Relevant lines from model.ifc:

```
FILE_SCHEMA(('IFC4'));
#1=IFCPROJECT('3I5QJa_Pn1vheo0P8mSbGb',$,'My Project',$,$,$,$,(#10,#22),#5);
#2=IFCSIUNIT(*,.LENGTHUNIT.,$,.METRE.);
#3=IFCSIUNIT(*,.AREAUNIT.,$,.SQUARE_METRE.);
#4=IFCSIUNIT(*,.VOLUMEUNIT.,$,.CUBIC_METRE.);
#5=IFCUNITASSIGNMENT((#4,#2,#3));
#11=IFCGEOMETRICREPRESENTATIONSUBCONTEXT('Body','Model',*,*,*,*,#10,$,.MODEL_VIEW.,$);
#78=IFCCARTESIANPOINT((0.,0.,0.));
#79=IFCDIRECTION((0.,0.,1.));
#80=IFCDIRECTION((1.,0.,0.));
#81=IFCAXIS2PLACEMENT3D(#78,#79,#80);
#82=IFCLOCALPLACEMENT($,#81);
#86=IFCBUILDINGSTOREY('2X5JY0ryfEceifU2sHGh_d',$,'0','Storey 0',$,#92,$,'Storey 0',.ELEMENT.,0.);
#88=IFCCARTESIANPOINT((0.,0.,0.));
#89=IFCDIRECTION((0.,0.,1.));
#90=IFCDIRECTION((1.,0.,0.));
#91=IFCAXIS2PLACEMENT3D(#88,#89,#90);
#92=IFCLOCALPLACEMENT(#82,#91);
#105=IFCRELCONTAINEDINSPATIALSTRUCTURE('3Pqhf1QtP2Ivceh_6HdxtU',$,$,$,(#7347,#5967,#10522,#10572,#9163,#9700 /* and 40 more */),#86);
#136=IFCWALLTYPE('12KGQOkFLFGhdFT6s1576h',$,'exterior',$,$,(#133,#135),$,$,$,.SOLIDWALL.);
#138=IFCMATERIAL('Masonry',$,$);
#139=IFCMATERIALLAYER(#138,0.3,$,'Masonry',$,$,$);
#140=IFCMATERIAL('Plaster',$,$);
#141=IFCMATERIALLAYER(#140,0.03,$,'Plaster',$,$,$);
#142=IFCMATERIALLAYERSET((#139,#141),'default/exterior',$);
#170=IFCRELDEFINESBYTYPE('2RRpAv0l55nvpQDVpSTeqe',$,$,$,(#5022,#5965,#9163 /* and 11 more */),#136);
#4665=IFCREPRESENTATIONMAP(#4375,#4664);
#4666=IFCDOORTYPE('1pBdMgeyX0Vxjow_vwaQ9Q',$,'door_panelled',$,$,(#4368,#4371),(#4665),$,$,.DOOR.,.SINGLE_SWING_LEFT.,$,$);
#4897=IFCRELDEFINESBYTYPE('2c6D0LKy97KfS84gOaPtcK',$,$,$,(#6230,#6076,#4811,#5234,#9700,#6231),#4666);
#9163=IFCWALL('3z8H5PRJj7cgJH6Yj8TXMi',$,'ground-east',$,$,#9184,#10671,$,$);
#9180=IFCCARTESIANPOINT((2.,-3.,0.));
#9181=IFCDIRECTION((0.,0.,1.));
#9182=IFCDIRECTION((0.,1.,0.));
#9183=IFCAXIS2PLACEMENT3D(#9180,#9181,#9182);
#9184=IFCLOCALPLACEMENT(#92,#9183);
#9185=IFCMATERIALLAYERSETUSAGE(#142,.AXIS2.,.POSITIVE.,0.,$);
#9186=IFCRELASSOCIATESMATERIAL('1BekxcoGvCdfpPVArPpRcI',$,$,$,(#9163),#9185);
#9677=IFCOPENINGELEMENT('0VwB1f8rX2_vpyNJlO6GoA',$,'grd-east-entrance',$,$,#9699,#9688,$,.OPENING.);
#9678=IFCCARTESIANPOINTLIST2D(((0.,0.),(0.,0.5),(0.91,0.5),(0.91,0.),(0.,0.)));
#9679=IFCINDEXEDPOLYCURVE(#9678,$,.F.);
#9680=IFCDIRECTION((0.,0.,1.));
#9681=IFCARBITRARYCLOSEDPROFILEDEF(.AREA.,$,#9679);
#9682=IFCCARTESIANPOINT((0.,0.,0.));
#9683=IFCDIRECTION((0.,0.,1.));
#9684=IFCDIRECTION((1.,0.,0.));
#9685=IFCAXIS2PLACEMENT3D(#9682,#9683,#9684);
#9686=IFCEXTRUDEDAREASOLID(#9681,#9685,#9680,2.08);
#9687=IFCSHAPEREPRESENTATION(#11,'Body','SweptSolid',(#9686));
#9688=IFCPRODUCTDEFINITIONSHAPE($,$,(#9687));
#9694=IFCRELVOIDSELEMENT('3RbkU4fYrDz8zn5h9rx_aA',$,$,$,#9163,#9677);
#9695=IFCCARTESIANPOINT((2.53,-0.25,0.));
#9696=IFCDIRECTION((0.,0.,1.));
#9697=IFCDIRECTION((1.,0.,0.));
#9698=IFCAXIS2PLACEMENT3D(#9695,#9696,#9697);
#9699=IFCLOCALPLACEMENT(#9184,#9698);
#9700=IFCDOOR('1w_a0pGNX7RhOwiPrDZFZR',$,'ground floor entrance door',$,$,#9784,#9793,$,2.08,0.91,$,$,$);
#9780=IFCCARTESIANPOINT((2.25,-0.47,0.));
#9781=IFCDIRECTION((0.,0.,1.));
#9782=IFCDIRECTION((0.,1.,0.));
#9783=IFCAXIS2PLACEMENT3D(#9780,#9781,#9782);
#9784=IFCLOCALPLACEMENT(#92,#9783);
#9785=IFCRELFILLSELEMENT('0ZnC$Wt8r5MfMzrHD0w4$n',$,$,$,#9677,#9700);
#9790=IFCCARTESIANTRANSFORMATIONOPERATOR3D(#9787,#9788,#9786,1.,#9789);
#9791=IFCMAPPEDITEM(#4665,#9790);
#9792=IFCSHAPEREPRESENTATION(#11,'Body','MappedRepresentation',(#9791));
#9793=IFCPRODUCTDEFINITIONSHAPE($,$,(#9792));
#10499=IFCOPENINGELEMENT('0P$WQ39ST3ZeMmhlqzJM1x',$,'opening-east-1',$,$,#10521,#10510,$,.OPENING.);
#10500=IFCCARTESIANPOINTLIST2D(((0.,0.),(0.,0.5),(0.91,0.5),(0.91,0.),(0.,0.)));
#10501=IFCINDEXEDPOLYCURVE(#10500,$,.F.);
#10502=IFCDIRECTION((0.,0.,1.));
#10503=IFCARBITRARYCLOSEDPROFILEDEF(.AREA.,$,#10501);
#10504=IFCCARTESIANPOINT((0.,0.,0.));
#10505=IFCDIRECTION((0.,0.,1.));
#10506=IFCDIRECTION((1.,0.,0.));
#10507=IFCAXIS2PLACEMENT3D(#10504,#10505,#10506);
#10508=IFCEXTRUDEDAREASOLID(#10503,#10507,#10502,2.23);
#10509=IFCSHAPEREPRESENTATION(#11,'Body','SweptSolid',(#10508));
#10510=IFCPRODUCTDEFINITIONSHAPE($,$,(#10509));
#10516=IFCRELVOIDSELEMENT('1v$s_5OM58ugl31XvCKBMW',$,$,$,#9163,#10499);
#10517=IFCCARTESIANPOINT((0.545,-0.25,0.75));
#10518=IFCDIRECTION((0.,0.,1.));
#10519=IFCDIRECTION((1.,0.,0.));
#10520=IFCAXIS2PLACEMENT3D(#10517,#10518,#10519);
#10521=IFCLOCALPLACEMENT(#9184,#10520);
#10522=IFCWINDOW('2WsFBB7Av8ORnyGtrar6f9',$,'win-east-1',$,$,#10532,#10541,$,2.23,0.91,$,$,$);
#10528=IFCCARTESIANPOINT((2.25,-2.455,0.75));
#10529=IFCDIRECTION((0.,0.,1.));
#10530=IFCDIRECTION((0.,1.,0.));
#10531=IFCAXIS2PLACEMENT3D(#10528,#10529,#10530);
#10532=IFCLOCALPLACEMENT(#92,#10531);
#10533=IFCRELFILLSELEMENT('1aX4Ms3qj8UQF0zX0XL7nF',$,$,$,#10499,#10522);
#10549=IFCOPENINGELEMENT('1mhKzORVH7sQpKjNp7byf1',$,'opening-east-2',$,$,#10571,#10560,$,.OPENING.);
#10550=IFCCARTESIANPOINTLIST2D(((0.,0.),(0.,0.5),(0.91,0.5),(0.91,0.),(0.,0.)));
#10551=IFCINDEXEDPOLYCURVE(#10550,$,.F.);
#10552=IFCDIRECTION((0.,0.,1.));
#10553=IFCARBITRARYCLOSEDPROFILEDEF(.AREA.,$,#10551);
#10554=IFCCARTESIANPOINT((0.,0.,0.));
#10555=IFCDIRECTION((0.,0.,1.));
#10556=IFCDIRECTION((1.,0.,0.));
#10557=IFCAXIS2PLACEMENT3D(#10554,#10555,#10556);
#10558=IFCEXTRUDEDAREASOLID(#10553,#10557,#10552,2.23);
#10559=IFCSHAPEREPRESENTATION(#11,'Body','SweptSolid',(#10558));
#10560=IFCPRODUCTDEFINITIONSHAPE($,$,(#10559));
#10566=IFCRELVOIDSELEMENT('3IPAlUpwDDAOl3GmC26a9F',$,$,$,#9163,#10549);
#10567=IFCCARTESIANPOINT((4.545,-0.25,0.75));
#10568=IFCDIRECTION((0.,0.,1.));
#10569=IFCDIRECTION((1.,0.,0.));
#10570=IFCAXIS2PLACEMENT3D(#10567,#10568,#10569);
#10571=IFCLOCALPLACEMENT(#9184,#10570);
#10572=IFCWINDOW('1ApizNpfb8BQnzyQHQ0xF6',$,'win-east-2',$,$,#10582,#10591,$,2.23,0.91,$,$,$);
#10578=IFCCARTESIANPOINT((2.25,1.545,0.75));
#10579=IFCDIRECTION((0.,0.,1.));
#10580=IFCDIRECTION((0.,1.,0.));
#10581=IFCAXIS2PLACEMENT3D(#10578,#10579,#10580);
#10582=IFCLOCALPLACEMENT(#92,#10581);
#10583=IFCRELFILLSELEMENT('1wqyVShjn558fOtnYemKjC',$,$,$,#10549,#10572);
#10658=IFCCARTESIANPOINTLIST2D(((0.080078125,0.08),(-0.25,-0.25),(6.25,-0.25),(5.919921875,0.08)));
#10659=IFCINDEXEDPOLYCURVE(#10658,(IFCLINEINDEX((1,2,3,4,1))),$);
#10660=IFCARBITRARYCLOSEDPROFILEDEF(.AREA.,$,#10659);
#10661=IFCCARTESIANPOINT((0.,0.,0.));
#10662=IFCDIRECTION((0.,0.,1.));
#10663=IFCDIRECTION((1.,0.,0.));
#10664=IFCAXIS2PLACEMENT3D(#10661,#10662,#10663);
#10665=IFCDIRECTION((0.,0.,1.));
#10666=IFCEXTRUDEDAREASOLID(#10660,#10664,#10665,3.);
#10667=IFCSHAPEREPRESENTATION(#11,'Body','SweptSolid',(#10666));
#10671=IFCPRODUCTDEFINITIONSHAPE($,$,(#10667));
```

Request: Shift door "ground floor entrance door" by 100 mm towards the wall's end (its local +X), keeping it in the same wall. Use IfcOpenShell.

```python
import ifcopenshell
import ifcopenshell.api.geometry
import ifcopenshell.util.placement
import ifcopenshell.util.unit

model = ifcopenshell.open("model.ifc")
unit_scale = ifcopenshell.util.unit.calculate_unit_scale(model)

door = model.by_id(9700)
opening = door.FillsVoids[0].RelatingOpeningElement
wall = opening.VoidsElements[0].RelatingBuildingElement

wall_matrix = ifcopenshell.util.placement.get_local_placement(wall.ObjectPlacement)
shift = wall_matrix[:3, 0] * 0.1 / unit_scale
before = ifcopenshell.util.placement.get_local_placement(door.ObjectPlacement)[:3, 3].copy()

# The door is not placed relative to its opening, so move both.
for product in (opening, door):
    matrix = ifcopenshell.util.placement.get_local_placement(product.ObjectPlacement)
    matrix[:3, 3] += shift
    ifcopenshell.api.geometry.edit_object_placement(model, product=product, matrix=matrix, is_si=False)

after = ifcopenshell.util.placement.get_local_placement(door.ObjectPlacement)[:3, 3]
print("door moved by", (after - before).round(3) + 0.0)

model.write("model_v2.ifc")
```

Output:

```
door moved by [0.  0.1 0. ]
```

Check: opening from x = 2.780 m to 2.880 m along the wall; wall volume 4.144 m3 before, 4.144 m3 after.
